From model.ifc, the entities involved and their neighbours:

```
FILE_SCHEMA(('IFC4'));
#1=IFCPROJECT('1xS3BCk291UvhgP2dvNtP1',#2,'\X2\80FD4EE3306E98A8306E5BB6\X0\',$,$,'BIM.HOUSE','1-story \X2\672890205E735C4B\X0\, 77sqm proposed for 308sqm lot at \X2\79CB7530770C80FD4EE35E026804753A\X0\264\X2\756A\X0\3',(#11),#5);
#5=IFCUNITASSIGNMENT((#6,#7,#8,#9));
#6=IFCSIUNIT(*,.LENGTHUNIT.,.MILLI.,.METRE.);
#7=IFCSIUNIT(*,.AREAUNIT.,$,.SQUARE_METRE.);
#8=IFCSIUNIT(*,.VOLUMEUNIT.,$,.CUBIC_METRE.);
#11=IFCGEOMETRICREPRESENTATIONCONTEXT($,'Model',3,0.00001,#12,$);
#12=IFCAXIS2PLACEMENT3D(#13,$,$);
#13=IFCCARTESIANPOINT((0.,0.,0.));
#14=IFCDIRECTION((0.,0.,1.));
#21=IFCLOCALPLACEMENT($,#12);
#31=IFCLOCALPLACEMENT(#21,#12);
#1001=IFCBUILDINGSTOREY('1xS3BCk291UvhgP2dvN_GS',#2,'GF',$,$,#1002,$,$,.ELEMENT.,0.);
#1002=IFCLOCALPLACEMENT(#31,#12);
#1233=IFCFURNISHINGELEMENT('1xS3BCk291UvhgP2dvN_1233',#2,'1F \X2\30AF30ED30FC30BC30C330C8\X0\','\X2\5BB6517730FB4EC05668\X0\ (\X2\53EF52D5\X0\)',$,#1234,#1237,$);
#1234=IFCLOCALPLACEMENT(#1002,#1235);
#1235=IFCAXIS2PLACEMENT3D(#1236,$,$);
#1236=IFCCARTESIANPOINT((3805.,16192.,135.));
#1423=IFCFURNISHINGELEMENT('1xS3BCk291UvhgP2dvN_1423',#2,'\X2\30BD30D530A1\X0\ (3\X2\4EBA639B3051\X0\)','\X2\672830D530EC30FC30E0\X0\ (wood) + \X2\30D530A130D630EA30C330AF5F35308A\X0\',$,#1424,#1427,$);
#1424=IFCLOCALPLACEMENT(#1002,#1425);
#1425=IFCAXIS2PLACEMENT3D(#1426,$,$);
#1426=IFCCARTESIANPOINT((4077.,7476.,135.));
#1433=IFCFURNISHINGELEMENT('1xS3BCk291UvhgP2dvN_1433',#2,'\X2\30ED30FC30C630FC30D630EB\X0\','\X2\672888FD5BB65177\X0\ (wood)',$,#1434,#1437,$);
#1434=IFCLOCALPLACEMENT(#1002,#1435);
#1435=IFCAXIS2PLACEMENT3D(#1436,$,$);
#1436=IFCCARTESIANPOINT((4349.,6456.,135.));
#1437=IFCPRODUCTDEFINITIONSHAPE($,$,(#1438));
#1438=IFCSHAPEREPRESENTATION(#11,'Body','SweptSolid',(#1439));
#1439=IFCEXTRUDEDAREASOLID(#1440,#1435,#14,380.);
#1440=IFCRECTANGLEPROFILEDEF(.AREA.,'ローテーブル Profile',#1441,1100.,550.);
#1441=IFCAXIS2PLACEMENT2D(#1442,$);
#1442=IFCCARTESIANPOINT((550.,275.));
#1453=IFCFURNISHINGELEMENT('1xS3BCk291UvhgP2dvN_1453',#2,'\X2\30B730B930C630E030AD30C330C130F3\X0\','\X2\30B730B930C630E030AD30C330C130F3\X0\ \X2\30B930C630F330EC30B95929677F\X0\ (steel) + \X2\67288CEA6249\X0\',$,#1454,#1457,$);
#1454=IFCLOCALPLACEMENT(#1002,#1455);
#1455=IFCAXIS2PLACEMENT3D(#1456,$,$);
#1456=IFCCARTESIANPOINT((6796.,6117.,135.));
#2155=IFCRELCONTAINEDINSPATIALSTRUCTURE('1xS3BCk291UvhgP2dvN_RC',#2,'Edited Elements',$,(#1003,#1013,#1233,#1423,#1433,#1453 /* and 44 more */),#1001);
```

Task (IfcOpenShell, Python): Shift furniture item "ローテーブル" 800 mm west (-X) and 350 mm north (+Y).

```python
import ifcopenshell
import ifcopenshell.api.geometry
import ifcopenshell.util.placement
import ifcopenshell.util.unit

model = ifcopenshell.open("model.ifc")
unit_scale = ifcopenshell.util.unit.calculate_unit_scale(model)

item = model.by_guid("1xS3BCk291UvhgP2dvN_1433")
matrix = ifcopenshell.util.placement.get_local_placement(item.ObjectPlacement)
matrix[0, 3] -= 0.8 / unit_scale
matrix[1, 3] += 0.35 / unit_scale
ifcopenshell.api.geometry.edit_object_placement(model, product=item, matrix=matrix, is_si=False)

print(ifcopenshell.util.placement.get_local_placement(item.ObjectPlacement).round(3) + 0.0)

model.write("model_edited.ifc")
```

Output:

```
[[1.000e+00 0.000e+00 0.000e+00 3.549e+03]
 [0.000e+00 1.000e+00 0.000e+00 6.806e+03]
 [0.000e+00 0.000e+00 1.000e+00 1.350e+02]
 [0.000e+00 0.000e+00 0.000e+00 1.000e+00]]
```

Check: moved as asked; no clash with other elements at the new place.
